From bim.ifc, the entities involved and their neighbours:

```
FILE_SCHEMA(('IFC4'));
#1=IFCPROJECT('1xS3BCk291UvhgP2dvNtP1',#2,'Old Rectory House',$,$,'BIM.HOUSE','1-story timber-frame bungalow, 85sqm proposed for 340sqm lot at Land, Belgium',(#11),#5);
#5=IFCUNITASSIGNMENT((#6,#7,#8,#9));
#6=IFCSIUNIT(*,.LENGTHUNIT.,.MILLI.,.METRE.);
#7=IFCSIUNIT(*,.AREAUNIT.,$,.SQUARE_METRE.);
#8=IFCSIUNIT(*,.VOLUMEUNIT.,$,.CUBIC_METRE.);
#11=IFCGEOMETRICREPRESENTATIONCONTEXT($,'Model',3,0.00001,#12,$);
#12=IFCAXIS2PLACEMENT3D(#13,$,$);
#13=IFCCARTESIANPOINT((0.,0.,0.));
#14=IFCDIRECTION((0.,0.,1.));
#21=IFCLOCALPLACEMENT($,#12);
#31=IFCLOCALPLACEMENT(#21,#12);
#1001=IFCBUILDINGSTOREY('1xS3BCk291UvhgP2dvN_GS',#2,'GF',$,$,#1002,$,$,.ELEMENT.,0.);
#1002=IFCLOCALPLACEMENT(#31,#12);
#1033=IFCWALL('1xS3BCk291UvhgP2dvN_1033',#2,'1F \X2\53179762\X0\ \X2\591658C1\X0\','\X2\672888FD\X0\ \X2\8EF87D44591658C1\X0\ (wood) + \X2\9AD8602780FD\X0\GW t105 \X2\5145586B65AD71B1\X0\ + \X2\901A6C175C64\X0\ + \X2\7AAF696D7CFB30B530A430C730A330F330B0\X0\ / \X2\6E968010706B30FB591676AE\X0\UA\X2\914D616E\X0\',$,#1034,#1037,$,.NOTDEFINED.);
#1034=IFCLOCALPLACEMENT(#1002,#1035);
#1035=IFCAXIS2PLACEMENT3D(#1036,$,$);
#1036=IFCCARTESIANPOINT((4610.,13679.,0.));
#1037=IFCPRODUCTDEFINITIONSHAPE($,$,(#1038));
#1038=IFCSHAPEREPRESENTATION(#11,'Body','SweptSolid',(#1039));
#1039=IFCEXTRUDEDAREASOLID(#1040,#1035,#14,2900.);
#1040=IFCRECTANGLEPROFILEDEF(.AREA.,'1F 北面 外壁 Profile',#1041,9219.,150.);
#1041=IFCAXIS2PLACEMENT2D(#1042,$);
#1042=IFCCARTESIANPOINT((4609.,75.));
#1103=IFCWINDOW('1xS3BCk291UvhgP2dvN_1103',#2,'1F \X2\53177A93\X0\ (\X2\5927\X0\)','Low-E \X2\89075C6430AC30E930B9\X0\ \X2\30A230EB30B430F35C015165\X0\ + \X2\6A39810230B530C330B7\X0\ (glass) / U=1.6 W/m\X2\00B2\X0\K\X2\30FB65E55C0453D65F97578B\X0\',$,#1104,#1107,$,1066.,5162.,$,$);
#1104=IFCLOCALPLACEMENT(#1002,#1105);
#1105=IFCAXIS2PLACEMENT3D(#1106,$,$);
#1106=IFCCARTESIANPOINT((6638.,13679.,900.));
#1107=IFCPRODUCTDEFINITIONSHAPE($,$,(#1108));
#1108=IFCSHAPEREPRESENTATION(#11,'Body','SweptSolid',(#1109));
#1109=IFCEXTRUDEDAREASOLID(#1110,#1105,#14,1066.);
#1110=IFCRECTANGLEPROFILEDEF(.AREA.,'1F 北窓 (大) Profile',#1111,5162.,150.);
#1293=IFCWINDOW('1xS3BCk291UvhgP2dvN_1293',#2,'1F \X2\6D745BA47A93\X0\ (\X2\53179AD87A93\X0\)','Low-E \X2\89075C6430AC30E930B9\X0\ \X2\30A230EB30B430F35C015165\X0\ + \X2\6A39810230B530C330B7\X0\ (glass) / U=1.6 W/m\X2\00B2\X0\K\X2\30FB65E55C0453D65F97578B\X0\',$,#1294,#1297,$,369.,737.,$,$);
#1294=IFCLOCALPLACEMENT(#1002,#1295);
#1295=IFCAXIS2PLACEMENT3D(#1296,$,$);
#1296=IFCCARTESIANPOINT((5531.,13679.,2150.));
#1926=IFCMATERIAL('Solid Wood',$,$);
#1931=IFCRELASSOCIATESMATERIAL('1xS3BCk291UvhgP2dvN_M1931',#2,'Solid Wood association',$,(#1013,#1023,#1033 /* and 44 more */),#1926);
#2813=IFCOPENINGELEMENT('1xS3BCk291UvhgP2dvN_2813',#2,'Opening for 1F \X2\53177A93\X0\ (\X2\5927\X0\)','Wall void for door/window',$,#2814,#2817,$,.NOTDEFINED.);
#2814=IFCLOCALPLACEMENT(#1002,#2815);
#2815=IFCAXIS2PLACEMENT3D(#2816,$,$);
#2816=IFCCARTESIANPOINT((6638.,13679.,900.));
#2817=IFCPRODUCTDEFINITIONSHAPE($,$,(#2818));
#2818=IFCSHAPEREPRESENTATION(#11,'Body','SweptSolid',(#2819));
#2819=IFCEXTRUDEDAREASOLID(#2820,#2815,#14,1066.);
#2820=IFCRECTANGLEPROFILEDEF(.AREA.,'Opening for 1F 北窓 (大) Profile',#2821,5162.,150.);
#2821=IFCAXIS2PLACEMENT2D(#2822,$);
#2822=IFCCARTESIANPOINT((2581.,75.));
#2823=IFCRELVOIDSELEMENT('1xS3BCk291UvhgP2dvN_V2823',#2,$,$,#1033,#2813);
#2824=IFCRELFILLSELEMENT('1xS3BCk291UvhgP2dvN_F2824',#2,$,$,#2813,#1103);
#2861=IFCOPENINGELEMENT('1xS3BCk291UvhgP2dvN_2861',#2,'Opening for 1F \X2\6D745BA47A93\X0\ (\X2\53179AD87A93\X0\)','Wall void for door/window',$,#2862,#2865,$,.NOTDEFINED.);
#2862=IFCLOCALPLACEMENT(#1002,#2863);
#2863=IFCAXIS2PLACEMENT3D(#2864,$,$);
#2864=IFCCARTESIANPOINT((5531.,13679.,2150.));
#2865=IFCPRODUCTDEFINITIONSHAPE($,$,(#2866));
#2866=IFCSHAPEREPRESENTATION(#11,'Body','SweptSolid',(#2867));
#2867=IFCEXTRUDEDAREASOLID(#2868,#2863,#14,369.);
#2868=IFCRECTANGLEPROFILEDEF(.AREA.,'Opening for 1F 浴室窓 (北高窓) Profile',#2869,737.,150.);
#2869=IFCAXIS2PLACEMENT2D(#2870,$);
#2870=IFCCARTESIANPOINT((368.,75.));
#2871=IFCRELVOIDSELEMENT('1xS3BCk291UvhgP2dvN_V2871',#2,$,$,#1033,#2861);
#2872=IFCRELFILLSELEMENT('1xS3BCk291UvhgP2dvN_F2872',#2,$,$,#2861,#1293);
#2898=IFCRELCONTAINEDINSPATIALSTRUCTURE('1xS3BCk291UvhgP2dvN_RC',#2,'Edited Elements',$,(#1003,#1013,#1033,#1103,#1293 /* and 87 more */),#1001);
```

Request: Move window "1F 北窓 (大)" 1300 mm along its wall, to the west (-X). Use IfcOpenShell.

```python
import ifcopenshell
import ifcopenshell.api.geometry
import ifcopenshell.util.placement
import ifcopenshell.util.unit

model = ifcopenshell.open("bim.ifc")
unit_scale = ifcopenshell.util.unit.calculate_unit_scale(model)

window = model.by_guid("1xS3BCk291UvhgP2dvN_1103")
opening = window.FillsVoids[0].RelatingOpeningElement
wall = opening.VoidsElements[0].RelatingBuildingElement

wall_matrix = ifcopenshell.util.placement.get_local_placement(wall.ObjectPlacement)
shift = wall_matrix[:3, 0] * -1.3 / unit_scale
before = ifcopenshell.util.placement.get_local_placement(window.ObjectPlacement)[:3, 3].copy()

# The window is not placed relative to its opening, so move both.
for product in (opening, window):
    matrix = ifcopenshell.util.placement.get_local_placement(product.ObjectPlacement)
    matrix[:3, 3] += shift
    ifcopenshell.api.geometry.edit_object_placement(model, product=product, matrix=matrix, is_si=False)

after = ifcopenshell.util.placement.get_local_placement(window.ObjectPlacement)[:3, 3]
print("window moved by", (after - before).round(3) + 0.0)

model.write("bim-out.ifc")
```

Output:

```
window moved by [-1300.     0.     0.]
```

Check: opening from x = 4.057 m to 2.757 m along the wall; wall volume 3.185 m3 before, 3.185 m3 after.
